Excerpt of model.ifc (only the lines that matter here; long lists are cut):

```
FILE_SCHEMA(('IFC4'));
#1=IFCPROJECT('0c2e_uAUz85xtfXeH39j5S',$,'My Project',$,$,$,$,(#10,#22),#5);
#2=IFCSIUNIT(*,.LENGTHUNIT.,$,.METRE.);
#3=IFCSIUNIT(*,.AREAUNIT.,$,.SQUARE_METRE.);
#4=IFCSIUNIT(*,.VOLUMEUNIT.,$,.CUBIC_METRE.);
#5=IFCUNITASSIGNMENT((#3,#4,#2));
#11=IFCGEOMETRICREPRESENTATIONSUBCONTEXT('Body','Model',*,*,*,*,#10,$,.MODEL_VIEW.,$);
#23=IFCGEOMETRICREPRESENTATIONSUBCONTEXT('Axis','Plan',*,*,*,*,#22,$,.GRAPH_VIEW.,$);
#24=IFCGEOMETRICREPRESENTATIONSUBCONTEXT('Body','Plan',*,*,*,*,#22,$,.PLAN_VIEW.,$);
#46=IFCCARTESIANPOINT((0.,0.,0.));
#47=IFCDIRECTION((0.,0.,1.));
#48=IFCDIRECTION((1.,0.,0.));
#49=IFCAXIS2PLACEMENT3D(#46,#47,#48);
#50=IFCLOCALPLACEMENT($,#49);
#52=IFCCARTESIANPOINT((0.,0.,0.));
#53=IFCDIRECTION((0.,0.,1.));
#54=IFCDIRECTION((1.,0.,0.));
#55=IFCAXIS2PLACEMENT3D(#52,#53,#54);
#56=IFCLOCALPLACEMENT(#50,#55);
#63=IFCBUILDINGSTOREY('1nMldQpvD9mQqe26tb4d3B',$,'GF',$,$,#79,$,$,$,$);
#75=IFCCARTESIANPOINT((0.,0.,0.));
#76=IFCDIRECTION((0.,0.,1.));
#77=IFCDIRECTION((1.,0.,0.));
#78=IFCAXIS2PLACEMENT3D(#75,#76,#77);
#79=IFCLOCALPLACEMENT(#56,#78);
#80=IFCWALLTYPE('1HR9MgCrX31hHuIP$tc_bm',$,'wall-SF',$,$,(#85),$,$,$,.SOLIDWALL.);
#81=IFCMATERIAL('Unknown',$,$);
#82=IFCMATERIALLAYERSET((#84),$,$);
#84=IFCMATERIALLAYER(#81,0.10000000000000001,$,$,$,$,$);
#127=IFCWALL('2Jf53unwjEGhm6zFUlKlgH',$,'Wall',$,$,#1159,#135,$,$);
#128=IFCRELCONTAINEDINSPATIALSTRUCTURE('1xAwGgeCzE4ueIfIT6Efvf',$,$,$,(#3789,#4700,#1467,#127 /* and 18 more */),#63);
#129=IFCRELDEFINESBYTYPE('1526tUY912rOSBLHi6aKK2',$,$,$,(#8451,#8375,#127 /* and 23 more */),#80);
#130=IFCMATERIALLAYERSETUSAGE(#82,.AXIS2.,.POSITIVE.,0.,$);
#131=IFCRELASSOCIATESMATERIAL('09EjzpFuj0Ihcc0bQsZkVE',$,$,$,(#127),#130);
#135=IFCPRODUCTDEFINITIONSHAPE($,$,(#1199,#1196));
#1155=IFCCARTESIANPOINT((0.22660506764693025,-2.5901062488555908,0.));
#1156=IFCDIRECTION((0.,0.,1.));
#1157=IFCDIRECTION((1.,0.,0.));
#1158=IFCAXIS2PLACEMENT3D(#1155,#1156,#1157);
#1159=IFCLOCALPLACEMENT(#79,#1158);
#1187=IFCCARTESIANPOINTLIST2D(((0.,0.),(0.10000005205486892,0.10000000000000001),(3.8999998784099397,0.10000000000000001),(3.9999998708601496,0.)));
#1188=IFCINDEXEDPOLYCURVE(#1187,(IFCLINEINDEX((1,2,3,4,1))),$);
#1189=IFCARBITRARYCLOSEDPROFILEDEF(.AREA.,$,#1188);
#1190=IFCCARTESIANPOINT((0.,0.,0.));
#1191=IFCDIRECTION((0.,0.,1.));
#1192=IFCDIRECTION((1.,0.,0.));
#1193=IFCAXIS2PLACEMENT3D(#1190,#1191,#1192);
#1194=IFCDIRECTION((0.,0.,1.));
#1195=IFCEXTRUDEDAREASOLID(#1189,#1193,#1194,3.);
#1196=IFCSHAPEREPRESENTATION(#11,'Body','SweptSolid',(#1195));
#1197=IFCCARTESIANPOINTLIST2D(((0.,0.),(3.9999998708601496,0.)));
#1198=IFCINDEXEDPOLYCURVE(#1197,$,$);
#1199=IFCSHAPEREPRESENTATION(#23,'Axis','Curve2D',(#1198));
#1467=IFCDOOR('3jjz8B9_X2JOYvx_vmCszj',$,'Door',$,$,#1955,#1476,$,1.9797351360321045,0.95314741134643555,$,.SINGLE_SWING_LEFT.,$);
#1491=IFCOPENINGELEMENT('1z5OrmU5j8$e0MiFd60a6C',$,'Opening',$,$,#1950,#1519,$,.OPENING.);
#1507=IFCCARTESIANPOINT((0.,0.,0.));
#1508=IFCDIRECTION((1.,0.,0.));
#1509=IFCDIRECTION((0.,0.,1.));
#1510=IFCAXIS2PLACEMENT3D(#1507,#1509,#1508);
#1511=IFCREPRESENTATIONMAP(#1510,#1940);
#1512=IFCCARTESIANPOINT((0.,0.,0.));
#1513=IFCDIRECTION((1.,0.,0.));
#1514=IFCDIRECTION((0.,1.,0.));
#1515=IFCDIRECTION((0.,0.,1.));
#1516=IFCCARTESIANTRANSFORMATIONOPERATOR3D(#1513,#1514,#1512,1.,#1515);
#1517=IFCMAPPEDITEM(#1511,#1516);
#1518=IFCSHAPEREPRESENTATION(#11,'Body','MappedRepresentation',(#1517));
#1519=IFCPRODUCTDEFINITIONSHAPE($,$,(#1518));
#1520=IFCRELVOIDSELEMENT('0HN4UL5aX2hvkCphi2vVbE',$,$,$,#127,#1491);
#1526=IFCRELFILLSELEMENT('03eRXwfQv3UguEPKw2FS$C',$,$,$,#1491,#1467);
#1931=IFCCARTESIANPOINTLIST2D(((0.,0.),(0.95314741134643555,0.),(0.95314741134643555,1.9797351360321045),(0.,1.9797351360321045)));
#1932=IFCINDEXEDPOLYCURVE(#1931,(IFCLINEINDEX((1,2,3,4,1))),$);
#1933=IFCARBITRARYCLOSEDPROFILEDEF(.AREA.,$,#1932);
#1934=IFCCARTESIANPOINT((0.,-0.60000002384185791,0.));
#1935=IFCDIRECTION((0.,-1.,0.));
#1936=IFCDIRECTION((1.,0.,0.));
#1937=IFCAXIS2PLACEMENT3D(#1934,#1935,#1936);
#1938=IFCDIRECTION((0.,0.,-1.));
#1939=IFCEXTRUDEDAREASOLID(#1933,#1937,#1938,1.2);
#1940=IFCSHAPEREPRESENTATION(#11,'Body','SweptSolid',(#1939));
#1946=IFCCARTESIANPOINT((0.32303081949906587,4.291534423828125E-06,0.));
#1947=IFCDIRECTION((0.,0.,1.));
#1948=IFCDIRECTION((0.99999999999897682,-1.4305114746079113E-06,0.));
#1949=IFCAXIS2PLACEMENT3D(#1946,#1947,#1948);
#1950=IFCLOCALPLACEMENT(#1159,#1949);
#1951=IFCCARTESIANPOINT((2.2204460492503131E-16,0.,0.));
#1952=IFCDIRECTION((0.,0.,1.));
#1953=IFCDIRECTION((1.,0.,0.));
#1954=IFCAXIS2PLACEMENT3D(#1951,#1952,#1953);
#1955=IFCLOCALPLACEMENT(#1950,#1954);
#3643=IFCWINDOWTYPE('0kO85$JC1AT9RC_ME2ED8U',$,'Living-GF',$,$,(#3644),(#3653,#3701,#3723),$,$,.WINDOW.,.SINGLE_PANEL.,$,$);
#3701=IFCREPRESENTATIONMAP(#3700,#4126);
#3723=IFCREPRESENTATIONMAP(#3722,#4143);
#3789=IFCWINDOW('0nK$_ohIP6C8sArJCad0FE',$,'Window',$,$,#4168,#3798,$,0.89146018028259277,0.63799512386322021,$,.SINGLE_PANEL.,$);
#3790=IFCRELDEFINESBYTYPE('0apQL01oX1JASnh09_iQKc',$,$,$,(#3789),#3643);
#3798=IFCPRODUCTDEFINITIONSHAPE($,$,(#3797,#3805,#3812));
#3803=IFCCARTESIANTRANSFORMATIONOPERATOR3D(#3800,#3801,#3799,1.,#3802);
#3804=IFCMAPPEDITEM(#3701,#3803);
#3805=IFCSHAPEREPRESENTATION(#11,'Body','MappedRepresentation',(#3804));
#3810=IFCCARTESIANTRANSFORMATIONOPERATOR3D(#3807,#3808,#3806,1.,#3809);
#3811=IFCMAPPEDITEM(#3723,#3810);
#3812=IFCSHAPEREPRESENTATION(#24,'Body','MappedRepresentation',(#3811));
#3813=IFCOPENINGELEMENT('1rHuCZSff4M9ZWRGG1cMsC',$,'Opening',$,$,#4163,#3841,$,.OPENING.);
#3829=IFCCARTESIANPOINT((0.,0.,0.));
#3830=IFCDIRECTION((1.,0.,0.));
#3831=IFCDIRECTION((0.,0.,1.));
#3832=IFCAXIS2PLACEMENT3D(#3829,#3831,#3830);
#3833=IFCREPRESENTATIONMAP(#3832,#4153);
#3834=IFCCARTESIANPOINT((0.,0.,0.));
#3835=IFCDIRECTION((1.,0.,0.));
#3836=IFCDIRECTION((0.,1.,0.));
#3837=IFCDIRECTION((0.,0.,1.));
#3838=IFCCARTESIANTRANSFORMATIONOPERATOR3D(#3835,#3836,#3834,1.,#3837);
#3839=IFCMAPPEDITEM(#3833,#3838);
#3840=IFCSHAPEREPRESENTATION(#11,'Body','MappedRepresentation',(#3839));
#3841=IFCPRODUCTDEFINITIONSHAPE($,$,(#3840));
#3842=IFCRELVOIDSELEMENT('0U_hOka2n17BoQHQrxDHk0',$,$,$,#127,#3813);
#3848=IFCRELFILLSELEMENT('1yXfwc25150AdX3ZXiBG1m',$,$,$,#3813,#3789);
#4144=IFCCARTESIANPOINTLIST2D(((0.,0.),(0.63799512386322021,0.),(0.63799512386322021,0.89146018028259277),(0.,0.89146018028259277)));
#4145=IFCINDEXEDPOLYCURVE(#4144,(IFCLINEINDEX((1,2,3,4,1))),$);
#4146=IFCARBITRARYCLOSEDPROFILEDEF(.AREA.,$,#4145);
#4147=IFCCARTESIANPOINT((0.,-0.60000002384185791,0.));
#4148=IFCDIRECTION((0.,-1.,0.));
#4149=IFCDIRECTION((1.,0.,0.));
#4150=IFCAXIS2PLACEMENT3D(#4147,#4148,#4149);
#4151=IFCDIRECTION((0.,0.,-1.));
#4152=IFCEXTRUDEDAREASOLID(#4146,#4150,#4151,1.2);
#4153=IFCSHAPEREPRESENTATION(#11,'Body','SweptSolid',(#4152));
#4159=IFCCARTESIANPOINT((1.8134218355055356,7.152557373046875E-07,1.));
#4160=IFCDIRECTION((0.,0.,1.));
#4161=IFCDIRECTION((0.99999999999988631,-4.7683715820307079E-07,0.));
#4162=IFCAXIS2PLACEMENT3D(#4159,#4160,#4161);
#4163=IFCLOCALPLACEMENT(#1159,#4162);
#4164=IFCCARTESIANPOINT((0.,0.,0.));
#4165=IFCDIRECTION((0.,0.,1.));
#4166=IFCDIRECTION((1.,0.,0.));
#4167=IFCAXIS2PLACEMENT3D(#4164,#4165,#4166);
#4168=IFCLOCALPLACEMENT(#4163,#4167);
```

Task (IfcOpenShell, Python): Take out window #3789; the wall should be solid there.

```python
import ifcopenshell
import ifcopenshell.api.feature
import ifcopenshell.api.root
import ifcopenshell.geom
import ifcopenshell.util.shape

model = ifcopenshell.open("model.ifc")
settings = ifcopenshell.geom.settings()


def volume(element):
    """Net volume in cubic metres, openings subtracted."""
    shape = ifcopenshell.geom.create_shape(settings, element)
    return ifcopenshell.util.shape.get_volume(shape.geometry)


window = model.by_guid("0nK$_ohIP6C8sArJCad0FE")
opening = window.FillsVoids[0].RelatingOpeningElement
wall = opening.VoidsElements[0].RelatingBuildingElement
before = volume(wall)

ifcopenshell.api.root.remove_product(model, product=window)
ifcopenshell.api.feature.remove_feature(model, feature=opening)

after = volume(wall)

print(f"wall volume {before:.3f} -> {after:.3f} m3")

model.write("model_edited.ifc")
```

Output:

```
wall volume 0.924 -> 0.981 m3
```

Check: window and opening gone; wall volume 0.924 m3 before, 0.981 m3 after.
